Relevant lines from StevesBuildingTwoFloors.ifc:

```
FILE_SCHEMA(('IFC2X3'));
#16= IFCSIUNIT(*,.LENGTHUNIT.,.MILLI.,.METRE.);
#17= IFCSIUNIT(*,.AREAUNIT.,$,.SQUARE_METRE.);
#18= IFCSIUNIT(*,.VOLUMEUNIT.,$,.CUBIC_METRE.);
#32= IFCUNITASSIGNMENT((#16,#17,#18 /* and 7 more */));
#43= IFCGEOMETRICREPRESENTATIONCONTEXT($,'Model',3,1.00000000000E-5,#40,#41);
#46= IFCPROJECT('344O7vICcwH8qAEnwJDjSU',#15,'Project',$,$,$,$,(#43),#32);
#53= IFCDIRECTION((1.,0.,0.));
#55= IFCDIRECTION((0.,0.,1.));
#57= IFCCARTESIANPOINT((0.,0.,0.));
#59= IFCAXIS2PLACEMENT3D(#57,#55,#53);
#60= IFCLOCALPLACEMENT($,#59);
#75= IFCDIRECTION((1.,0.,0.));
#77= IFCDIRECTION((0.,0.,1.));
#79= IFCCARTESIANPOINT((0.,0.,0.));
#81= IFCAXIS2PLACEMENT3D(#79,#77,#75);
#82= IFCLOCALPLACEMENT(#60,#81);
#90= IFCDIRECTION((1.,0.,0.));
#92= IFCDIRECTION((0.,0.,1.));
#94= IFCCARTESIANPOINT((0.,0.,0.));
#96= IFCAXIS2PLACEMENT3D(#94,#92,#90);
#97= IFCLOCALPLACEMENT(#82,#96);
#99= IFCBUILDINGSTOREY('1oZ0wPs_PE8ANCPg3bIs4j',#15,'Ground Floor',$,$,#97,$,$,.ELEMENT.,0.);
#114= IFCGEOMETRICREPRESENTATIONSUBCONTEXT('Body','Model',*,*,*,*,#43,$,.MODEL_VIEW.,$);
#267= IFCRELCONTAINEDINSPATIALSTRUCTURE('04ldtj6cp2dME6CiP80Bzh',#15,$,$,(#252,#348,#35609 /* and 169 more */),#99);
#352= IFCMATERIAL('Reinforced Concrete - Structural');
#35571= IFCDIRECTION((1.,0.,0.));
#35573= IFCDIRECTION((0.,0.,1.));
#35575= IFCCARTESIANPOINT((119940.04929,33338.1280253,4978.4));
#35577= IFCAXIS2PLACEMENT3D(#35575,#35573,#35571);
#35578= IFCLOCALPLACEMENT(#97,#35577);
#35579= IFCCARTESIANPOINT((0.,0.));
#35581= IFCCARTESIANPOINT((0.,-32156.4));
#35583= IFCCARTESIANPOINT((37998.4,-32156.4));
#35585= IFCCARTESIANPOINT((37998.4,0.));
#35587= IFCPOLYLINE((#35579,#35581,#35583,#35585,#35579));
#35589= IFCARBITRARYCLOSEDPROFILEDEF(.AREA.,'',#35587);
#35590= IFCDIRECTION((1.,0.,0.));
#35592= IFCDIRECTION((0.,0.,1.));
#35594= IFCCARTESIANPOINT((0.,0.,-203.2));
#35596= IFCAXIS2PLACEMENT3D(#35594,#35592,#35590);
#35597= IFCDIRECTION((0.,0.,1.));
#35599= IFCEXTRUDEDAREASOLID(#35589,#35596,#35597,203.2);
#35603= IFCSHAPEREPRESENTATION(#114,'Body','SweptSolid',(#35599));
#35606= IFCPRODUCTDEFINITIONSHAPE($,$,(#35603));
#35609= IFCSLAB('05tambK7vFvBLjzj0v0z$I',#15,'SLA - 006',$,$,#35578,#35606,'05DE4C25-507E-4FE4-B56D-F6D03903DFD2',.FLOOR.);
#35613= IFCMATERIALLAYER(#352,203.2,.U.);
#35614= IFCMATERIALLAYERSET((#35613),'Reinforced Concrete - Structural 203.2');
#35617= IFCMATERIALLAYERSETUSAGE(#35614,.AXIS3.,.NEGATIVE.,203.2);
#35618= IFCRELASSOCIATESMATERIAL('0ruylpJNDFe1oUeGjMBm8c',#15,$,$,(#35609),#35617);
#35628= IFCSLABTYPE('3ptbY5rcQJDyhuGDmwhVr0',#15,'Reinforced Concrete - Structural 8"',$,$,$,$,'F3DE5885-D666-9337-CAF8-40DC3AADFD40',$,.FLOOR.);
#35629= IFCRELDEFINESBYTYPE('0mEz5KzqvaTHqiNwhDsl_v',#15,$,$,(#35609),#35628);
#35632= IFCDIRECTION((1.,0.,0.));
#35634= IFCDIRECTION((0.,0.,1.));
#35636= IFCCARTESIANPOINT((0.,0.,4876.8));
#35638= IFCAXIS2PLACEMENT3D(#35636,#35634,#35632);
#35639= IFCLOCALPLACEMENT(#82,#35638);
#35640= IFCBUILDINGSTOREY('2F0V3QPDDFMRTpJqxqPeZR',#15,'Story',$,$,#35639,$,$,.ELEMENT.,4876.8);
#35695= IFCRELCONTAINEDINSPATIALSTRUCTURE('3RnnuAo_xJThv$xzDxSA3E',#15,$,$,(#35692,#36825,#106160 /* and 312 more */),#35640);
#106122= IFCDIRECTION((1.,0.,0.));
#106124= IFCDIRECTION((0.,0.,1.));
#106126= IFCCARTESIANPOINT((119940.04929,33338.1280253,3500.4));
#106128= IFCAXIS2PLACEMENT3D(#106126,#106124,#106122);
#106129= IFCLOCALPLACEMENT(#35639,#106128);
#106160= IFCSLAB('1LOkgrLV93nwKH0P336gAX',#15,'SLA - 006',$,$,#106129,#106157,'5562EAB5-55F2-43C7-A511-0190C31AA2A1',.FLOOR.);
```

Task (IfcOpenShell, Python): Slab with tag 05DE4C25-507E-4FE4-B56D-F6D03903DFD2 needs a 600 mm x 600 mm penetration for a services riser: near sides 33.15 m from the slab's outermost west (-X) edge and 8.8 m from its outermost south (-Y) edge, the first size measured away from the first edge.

```python
import numpy as np
import ifcopenshell
import ifcopenshell.api.feature
import ifcopenshell.api.geometry
import ifcopenshell.api.root
import ifcopenshell.geom
import ifcopenshell.util.placement
import ifcopenshell.util.representation
import ifcopenshell.util.shape
import ifcopenshell.util.unit

model = ifcopenshell.open("StevesBuildingTwoFloors.ifc")
unit_scale = ifcopenshell.util.unit.calculate_unit_scale(model)
settings = ifcopenshell.geom.settings()


def volume(element):
    """Net volume in cubic metres, openings subtracted."""
    shape = ifcopenshell.geom.create_shape(settings, element)
    return ifcopenshell.util.shape.get_volume(shape.geometry)


slab = model.by_id(35609)
before = volume(slab)

# Extent in the slab's own axes, in metres. The edges named are its -X and -Y sides.
slab_shape = ifcopenshell.geom.create_shape(settings, slab)
vertices = ifcopenshell.util.shape.get_vertices(slab_shape.geometry)
x_min, y_min, bottom = vertices.min(axis=0)
top = vertices[:, 2].max()

opening = ifcopenshell.api.root.create_entity(model, ifc_class="IfcOpeningElement", name="Services riser opening")
context = ifcopenshell.util.representation.get_context(model, "Model", "Body", "MODEL_VIEW")
width, depth = 0.6, 0.6
outline = [(0.0, 0.0), (width, 0.0), (width, depth), (0.0, depth), (0.0, 0.0)]
# Overshoot both faces by 50 mm so the cut is clean.
shape = ifcopenshell.api.geometry.add_slab_representation(
    model, context=context, depth=top - bottom + 0.1, polyline=outline
)
ifcopenshell.api.geometry.assign_representation(model, product=opening, representation=shape)

matrix = ifcopenshell.util.placement.get_local_placement(slab.ObjectPlacement)
matrix[:, 3] = matrix @ np.append(np.array([x_min + 33.15, y_min + 8.8, bottom - 0.05]) / unit_scale, 1.0)
ifcopenshell.api.geometry.edit_object_placement(model, product=opening, matrix=matrix, is_si=False)
ifcopenshell.api.feature.add_feature(model, feature=opening, element=slab)

after = volume(slab)

print(f"slab volume {before:.3f} -> {after:.3f} m3")

model.write("StevesBuildingTwoFloors_rev.ifc")
```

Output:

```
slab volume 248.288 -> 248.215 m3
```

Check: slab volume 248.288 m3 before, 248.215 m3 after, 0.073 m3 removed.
